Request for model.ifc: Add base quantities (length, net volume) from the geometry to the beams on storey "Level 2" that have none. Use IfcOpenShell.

First a look at what the model holds.

```python
import ifcopenshell
import ifcopenshell.util.element
import ifcopenshell.util.unit

model = ifcopenshell.open("model.ifc")
print(model.schema)
for unit_type in ("LENGTHUNIT", "AREAUNIT", "VOLUMEUNIT"):
    print(unit_type, ifcopenshell.util.unit.calculate_unit_scale(model, unit_type))
storey = next(s for s in model.by_type("IfcBuildingStorey") if s.Name == "Level 2")
beams = [e for e in ifcopenshell.util.element.get_decomposition(storey) if e.is_a("IfcBeam")]
for e in sorted(beams, key=lambda e: e.id()):
    print(e.id(), e.is_a(), e.Name, list(ifcopenshell.util.element.get_psets(e, qtos_only=True)), sep=" | ")
```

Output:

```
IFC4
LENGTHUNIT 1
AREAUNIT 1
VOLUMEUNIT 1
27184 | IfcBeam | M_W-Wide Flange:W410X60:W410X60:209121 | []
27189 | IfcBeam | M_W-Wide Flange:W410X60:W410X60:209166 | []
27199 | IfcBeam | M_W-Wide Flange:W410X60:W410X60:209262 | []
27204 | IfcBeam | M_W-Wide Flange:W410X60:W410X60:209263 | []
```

```python
import ifcopenshell
import ifcopenshell.api.pset
import ifcopenshell.geom
import ifcopenshell.util.element
import ifcopenshell.util.shape
import ifcopenshell.util.unit

model = ifcopenshell.open("model.ifc")
unit_scale = ifcopenshell.util.unit.calculate_unit_scale(model)
volume_scale = ifcopenshell.util.unit.calculate_unit_scale(model, "VOLUMEUNIT")
settings = ifcopenshell.geom.settings()

storey = next(s for s in model.by_type("IfcBuildingStorey") if s.Name == "Level 2")
beams = [e for e in ifcopenshell.util.element.get_decomposition(storey) if e.is_a("IfcBeam")]

for e in sorted(beams, key=lambda e: e.id()):
    if ifcopenshell.util.element.get_psets(e, qtos_only=True, should_inherit=False):
        continue
    # Geometry comes back in metres, in the element's own axes.
    shape = ifcopenshell.geom.create_shape(settings, e)
    values = {
        "Length": ifcopenshell.util.shape.get_max_xyz(shape.geometry) / unit_scale,
        "NetVolume": ifcopenshell.util.shape.get_volume(shape.geometry) / volume_scale,
    }
    qto = ifcopenshell.api.pset.add_qto(model, product=e, name="Qto_BeamBaseQuantities")
    ifcopenshell.api.pset.edit_qto(model, qto=qto, properties=values)
    print(e.id(), {k: round(v, 3) for k, v in values.items()})

model.write("model-out.ifc")
```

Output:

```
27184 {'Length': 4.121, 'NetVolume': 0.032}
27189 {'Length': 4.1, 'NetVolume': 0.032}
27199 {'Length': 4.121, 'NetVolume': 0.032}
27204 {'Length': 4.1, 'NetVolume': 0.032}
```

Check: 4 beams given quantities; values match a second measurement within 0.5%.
